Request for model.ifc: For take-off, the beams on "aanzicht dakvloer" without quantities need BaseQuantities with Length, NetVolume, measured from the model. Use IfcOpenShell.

First a look at what the model holds.

```python
import ifcopenshell
import ifcopenshell.util.element
import ifcopenshell.util.unit

model = ifcopenshell.open("model.ifc")
print(model.schema)
for unit_type in ("LENGTHUNIT", "AREAUNIT", "VOLUMEUNIT"):
    print(unit_type, ifcopenshell.util.unit.calculate_unit_scale(model, unit_type))
storey = next(s for s in model.by_type("IfcBuildingStorey") if s.Name == "aanzicht dakvloer")
beams = [e for e in ifcopenshell.util.element.get_decomposition(storey) if e.is_a("IfcBeam")]
for e in sorted(beams, key=lambda e: e.id()):
    print(e.id(), e.is_a(), e.Name, list(ifcopenshell.util.element.get_psets(e, qtos_only=True)), sep=" | ")
```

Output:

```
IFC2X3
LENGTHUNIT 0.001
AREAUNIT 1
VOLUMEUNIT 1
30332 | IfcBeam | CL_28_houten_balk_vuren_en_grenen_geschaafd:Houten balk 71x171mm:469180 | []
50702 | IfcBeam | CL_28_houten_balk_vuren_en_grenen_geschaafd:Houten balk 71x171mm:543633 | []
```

```python
import ifcopenshell
import ifcopenshell.api.pset
import ifcopenshell.geom
import ifcopenshell.util.element
import ifcopenshell.util.shape
import ifcopenshell.util.unit

model = ifcopenshell.open("model.ifc")
unit_scale = ifcopenshell.util.unit.calculate_unit_scale(model)
volume_scale = ifcopenshell.util.unit.calculate_unit_scale(model, "VOLUMEUNIT")
settings = ifcopenshell.geom.settings()

storey = next(s for s in model.by_type("IfcBuildingStorey") if s.Name == "aanzicht dakvloer")
beams = [e for e in ifcopenshell.util.element.get_decomposition(storey) if e.is_a("IfcBeam")]

for e in sorted(beams, key=lambda e: e.id()):
    if ifcopenshell.util.element.get_psets(e, qtos_only=True, should_inherit=False):
        continue
    # Geometry comes back in metres, in the element's own axes.
    shape = ifcopenshell.geom.create_shape(settings, e)
    values = {
        "Length": ifcopenshell.util.shape.get_max_xyz(shape.geometry) / unit_scale,
        "NetVolume": ifcopenshell.util.shape.get_volume(shape.geometry) / volume_scale,
    }
    qto = ifcopenshell.api.pset.add_qto(model, product=e, name="BaseQuantities")
    ifcopenshell.api.pset.edit_qto(model, qto=qto, properties=values)
    print(e.id(), {k: round(v, 3) for k, v in values.items()})

model.write("model_edited.ifc")
```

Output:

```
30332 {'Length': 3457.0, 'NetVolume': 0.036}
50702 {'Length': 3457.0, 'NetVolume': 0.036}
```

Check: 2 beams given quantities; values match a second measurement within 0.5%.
